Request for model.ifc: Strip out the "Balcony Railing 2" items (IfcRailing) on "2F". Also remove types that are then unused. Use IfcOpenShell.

First a look at what the model holds.

```python
import ifcopenshell
import ifcopenshell.util.element

model = ifcopenshell.open("model.ifc")
print(model.schema)
storey = next(s for s in model.by_type("IfcBuildingStorey") if s.Name == "2F")
railings = [e for e in ifcopenshell.util.element.get_decomposition(storey) if e.is_a("IfcRailing")]
seen = {}
for e in railings:
    element_type = ifcopenshell.util.element.get_type(e)
    name = element_type.Name if element_type not in (None, e) else None
    seen[name] = seen.get(name, 0) + 1
for name, count in sorted(seen.items(), key=str):
    print(count, "x", name)
```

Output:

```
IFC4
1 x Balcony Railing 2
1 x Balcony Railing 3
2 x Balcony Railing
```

```python
import ifcopenshell
import ifcopenshell.api.root
import ifcopenshell.util.element

model = ifcopenshell.open("model.ifc")

storey = next(s for s in model.by_type("IfcBuildingStorey") if s.Name == "2F")
railings = [e for e in ifcopenshell.util.element.get_decomposition(storey) if e.is_a("IfcRailing")]
targets = [e for e in railings if (t := ifcopenshell.util.element.get_type(e)) not in (None, e) and t.Name == "Balcony Railing 2"]
types = {ifcopenshell.util.element.get_type(e) for e in targets} - {None, *targets}

for e in targets:
    ifcopenshell.api.root.remove_product(model, product=e)
print(len(targets), "removed")

unused = [t for t in types if not ifcopenshell.util.element.get_types(t)]
for t in unused:
    ifcopenshell.api.root.remove_product(model, product=t)
print(len(unused), "unused types removed")

model.write("model_v2.ifc")
```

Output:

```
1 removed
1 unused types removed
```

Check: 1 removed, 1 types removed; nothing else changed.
